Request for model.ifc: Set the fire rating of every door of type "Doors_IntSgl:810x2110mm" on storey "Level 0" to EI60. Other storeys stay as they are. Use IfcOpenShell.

First a look at what the model holds.

```python
import ifcopenshell
import ifcopenshell.util.element

model = ifcopenshell.open("model.ifc")
print(model.schema)
storey = next(s for s in model.by_type("IfcBuildingStorey") if s.Name == "Level 0")
doors = [e for e in ifcopenshell.util.element.get_decomposition(storey) if e.is_a("IfcDoor")]
seen = {}
for e in doors:
    element_type = ifcopenshell.util.element.get_type(e)
    key = (element_type.Name if element_type != e and element_type else None, ifcopenshell.util.element.get_pset(e, "Pset_DoorCommon", "FireRating"))
    seen[key] = seen.get(key, 0) + 1
for (name, value), count in sorted(seen.items(), key=str):
    print(count, "x", name, "|", value)
```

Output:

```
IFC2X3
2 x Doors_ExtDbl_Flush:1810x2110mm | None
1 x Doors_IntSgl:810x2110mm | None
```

```python
import ifcopenshell
import ifcopenshell.api.pset
import ifcopenshell.util.element

model = ifcopenshell.open("model.ifc")

storey = next(s for s in model.by_type("IfcBuildingStorey") if s.Name == "Level 0")
doors = [e for e in ifcopenshell.util.element.get_decomposition(storey) if e.is_a("IfcDoor")]

count = 0
for e in doors:
    element_type = ifcopenshell.util.element.get_type(e)
    if element_type in (None, e) or element_type.Name != "Doors_IntSgl:810x2110mm":
        continue
    # add_pset returns the element's existing set when there is one.
    pset = ifcopenshell.api.pset.add_pset(model, product=e, name="Pset_DoorCommon")
    ifcopenshell.api.pset.edit_pset(model, pset=pset, properties={"FireRating": "EI60"})
    count += 1

print(count, "doors updated")

model.write("model-out.ifc")
```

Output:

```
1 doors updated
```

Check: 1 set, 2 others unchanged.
